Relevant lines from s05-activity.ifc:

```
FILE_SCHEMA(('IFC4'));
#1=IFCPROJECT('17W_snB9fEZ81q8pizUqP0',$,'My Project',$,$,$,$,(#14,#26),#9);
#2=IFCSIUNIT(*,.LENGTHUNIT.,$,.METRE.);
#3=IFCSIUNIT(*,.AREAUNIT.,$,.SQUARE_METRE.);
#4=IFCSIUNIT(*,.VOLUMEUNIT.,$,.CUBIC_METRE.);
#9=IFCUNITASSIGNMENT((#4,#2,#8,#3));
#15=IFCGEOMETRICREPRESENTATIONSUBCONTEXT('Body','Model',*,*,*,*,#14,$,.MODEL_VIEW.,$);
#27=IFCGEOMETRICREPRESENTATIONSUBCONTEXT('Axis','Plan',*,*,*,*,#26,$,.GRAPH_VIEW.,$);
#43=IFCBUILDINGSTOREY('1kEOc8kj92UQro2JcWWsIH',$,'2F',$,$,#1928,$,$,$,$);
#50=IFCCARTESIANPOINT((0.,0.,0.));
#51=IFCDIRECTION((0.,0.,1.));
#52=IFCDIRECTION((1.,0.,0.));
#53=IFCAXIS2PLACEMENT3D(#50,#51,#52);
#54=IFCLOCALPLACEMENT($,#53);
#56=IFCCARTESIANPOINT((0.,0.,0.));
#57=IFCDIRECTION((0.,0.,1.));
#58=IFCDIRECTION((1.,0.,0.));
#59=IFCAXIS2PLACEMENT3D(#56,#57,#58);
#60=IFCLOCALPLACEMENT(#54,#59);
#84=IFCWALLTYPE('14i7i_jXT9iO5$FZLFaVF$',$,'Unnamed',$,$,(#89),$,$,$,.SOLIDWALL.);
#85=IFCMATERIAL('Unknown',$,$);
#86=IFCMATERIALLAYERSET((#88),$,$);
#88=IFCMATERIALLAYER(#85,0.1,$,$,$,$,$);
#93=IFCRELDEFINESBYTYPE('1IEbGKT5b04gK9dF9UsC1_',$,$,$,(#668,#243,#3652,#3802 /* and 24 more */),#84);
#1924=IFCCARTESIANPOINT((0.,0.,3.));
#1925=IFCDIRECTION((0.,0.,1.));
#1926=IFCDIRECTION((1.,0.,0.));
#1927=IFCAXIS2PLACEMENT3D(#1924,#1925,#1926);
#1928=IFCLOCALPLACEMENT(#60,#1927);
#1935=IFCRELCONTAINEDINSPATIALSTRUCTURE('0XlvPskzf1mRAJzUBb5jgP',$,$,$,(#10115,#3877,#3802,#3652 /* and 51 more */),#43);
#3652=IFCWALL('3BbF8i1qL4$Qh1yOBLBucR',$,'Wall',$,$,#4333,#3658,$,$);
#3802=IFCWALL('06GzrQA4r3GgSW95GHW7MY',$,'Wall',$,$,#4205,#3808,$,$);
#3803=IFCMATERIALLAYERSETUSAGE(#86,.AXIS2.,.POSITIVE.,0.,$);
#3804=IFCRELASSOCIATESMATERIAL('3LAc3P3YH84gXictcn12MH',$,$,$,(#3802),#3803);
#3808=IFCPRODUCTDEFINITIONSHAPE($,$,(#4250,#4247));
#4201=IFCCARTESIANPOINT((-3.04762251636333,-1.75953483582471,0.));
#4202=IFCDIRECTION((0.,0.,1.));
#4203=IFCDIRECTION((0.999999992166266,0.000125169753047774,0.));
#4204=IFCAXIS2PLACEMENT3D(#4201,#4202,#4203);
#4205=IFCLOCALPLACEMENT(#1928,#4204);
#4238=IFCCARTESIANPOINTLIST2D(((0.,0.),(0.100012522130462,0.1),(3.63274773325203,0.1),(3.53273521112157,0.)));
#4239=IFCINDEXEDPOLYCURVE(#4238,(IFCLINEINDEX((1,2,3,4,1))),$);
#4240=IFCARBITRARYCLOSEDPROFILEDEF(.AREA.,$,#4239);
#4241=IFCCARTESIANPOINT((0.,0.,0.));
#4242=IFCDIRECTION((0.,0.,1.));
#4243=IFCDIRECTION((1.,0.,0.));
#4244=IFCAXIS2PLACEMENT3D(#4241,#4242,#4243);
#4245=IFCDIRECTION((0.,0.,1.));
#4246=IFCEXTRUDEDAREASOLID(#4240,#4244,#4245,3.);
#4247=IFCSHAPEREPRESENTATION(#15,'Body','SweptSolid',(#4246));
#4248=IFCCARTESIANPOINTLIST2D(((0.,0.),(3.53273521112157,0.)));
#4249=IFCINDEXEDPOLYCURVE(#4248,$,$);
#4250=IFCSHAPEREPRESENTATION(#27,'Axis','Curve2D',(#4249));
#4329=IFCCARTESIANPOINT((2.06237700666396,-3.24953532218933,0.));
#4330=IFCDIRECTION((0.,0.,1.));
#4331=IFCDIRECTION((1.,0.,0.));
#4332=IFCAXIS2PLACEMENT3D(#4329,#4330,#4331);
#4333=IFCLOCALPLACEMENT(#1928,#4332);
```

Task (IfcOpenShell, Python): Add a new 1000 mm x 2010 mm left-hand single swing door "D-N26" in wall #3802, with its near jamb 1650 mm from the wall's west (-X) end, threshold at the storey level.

```python
import numpy as np
import ifcopenshell
import ifcopenshell.api.feature
import ifcopenshell.api.geometry
import ifcopenshell.api.root
import ifcopenshell.api.spatial
import ifcopenshell.geom
import ifcopenshell.util.element
import ifcopenshell.util.placement
import ifcopenshell.util.representation
import ifcopenshell.util.shape
import ifcopenshell.util.unit

model = ifcopenshell.open("s05-activity.ifc")
unit_scale = ifcopenshell.util.unit.calculate_unit_scale(model)
settings = ifcopenshell.geom.settings()


def volume(element):
    """Net volume in cubic metres, openings subtracted."""
    shape = ifcopenshell.geom.create_shape(settings, element)
    return ifcopenshell.util.shape.get_volume(shape.geometry)


wall = model.by_guid("06GzrQA4r3GgSW95GHW7MY")
storey = ifcopenshell.util.element.get_container(wall, ifc_class="IfcBuildingStorey")
context = ifcopenshell.util.representation.get_context(model, "Model", "Body", "MODEL_VIEW")
before = volume(wall)

width, height, from_end, sill = 1, 2.01, 1.65, 0.0  # metres

# The wall runs along its own X axis, and the end named is its -X end.
wall_shape = ifcopenshell.geom.create_shape(settings, wall)
x, y, z = ifcopenshell.util.shape.get_vertices(wall_shape.geometry).T
start = x.min() + from_end
face, thickness = float(y.min()), float(y.max() - y.min())
wall_matrix = ifcopenshell.util.placement.get_local_placement(wall.ObjectPlacement)
level = ifcopenshell.util.placement.get_local_placement(storey.ObjectPlacement)[2, 3]


def in_wall(x, y):
    """Placement at x, y metres in the wall's axes, at sill height."""
    matrix = wall_matrix.copy()
    matrix[:, 3] = wall_matrix @ np.array([x / unit_scale, y / unit_scale, 0.0, 1.0])
    matrix[2, 3] = level + sill / unit_scale
    return matrix


# Opening: a box that overshoots both wall faces by 50 mm.
opening = ifcopenshell.api.root.create_entity(model, ifc_class="IfcOpeningElement", predefined_type="OPENING")
box = ifcopenshell.api.geometry.add_wall_representation(
    model, context=context, length=width, height=height, thickness=thickness + 0.1
)
ifcopenshell.api.geometry.assign_representation(model, product=opening, representation=box)
ifcopenshell.api.geometry.edit_object_placement(model, product=opening, matrix=in_wall(start, face - 0.05), is_si=False)
ifcopenshell.api.feature.add_feature(model, feature=opening, element=wall)

door = ifcopenshell.api.root.create_entity(model, ifc_class="IfcDoor", name="D-N26", predefined_type="DOOR")
door.OverallWidth, door.OverallHeight = width / unit_scale, height / unit_scale
door.OperationType = "SINGLE_SWING_LEFT"
body = ifcopenshell.api.geometry.add_door_representation(
    model,
    context=context,
    overall_width=door.OverallWidth,
    overall_height=door.OverallHeight,
    operation_type="SINGLE_SWING_LEFT",
    lining_properties={"LiningDepth": thickness / unit_scale, "ThresholdDepth": thickness / unit_scale},
)
ifcopenshell.api.geometry.assign_representation(model, product=door, representation=body)
ifcopenshell.api.spatial.assign_container(model, products=[door], relating_structure=storey)
ifcopenshell.api.feature.add_filling(model, opening=opening, element=door)

# The lining spans the wall, so the door starts at the wall face.
ifcopenshell.api.geometry.edit_object_placement(model, product=door, matrix=in_wall(start, face), is_si=False)

after = volume(wall)

print(f"wall volume {before:.3f} -> {after:.3f} m3")

model.write("s05-activity_v2.ifc")
```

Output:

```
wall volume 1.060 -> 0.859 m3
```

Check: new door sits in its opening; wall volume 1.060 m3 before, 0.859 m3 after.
